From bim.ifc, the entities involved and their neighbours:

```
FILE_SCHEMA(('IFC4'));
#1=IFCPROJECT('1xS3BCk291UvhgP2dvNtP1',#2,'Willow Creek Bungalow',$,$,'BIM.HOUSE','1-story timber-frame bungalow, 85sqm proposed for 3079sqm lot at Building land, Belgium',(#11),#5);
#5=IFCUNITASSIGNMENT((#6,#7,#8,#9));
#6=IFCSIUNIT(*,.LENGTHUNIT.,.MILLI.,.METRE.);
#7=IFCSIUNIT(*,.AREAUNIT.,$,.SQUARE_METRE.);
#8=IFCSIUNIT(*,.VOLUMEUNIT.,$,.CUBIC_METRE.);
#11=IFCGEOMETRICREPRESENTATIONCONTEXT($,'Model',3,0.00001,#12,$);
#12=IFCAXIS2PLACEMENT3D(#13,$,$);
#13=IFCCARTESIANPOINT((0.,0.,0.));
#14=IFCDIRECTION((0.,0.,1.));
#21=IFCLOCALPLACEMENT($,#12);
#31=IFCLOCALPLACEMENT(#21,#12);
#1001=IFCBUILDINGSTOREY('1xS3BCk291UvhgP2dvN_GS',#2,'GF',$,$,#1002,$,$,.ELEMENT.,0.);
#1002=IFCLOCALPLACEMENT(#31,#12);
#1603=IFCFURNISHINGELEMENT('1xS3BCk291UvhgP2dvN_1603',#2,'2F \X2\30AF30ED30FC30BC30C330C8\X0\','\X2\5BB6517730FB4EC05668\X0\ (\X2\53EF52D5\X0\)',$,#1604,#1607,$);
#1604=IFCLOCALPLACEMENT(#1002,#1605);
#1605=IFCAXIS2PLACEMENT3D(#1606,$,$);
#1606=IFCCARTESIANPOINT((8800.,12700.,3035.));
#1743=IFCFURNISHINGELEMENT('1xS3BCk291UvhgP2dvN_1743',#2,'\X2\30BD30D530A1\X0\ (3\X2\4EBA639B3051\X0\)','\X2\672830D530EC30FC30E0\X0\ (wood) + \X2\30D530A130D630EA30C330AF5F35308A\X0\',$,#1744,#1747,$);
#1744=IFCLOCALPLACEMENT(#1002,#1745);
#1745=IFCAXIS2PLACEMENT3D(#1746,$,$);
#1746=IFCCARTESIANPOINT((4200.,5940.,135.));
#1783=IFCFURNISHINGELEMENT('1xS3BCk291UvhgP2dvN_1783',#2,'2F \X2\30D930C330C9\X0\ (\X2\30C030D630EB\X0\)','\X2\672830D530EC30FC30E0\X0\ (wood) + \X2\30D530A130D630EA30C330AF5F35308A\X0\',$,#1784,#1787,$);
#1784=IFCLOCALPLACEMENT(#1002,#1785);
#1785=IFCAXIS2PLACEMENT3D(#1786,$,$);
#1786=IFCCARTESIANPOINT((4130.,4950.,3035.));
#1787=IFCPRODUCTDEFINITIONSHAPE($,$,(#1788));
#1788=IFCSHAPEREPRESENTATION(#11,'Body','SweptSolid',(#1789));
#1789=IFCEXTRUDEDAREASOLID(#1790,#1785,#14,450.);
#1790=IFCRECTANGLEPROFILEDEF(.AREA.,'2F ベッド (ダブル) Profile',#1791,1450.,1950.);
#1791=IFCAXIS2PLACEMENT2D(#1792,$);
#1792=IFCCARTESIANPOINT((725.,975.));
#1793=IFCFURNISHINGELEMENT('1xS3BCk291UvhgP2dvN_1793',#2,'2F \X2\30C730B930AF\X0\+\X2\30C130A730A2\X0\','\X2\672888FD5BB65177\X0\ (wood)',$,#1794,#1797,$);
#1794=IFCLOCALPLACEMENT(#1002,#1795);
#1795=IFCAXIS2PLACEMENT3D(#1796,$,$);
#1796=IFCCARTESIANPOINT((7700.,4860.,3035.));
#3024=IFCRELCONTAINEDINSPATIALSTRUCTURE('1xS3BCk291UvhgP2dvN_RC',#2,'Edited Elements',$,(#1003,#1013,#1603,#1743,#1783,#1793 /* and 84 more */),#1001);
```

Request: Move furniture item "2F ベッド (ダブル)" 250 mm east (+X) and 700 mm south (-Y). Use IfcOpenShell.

```python
import ifcopenshell
import ifcopenshell.api.geometry
import ifcopenshell.util.placement

model = ifcopenshell.open("bim.ifc")

item = model.by_guid("1xS3BCk291UvhgP2dvN_1783")
matrix = ifcopenshell.util.placement.get_local_placement(item.ObjectPlacement)
matrix[0, 3] += 250.0
matrix[1, 3] -= 700.0
ifcopenshell.api.geometry.edit_object_placement(model, product=item, matrix=matrix, is_si=False)

print(ifcopenshell.util.placement.get_local_placement(item.ObjectPlacement).round(3) + 0.0)

model.write("bim_v2.ifc")
```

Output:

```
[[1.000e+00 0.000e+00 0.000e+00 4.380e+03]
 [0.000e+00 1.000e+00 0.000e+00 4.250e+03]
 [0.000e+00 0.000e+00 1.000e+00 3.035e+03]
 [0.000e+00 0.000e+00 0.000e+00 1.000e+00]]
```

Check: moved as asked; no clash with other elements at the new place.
